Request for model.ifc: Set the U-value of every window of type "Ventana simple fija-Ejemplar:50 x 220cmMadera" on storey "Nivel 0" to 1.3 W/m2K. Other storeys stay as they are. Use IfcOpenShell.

First a look at what the model holds.

```python
import ifcopenshell
import ifcopenshell.util.element

model = ifcopenshell.open("model.ifc")
print(model.schema)
storey = next(s for s in model.by_type("IfcBuildingStorey") if s.Name == "Nivel 0")
windows = [e for e in ifcopenshell.util.element.get_decomposition(storey) if e.is_a("IfcWindow")]
seen = {}
for e in windows:
    element_type = ifcopenshell.util.element.get_type(e)
    key = (element_type.Name if element_type != e and element_type else None, ifcopenshell.util.element.get_pset(e, "Pset_WindowCommon", "ThermalTransmittance"))
    seen[key] = seen.get(key, 0) + 1
for (name, value), count in sorted(seen.items(), key=str):
    print(count, "x", name, "|", value)
```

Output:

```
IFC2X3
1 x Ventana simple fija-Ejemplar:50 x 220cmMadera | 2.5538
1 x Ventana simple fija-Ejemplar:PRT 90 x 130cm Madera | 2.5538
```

```python
import ifcopenshell
import ifcopenshell.api.pset
import ifcopenshell.util.element

model = ifcopenshell.open("model.ifc")

storey = next(s for s in model.by_type("IfcBuildingStorey") if s.Name == "Nivel 0")
windows = [e for e in ifcopenshell.util.element.get_decomposition(storey) if e.is_a("IfcWindow")]

count = 0
for e in windows:
    element_type = ifcopenshell.util.element.get_type(e)
    if element_type in (None, e) or element_type.Name != "Ventana simple fija-Ejemplar:50 x 220cmMadera":
        continue
    # add_pset returns the element's existing set when there is one.
    pset = ifcopenshell.api.pset.add_pset(model, product=e, name="Pset_WindowCommon")
    ifcopenshell.api.pset.edit_pset(model, pset=pset, properties={"ThermalTransmittance": 1.3})
    count += 1

print(count, "windows updated")

model.write("model_updated.ifc")
```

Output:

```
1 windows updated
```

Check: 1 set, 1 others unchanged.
